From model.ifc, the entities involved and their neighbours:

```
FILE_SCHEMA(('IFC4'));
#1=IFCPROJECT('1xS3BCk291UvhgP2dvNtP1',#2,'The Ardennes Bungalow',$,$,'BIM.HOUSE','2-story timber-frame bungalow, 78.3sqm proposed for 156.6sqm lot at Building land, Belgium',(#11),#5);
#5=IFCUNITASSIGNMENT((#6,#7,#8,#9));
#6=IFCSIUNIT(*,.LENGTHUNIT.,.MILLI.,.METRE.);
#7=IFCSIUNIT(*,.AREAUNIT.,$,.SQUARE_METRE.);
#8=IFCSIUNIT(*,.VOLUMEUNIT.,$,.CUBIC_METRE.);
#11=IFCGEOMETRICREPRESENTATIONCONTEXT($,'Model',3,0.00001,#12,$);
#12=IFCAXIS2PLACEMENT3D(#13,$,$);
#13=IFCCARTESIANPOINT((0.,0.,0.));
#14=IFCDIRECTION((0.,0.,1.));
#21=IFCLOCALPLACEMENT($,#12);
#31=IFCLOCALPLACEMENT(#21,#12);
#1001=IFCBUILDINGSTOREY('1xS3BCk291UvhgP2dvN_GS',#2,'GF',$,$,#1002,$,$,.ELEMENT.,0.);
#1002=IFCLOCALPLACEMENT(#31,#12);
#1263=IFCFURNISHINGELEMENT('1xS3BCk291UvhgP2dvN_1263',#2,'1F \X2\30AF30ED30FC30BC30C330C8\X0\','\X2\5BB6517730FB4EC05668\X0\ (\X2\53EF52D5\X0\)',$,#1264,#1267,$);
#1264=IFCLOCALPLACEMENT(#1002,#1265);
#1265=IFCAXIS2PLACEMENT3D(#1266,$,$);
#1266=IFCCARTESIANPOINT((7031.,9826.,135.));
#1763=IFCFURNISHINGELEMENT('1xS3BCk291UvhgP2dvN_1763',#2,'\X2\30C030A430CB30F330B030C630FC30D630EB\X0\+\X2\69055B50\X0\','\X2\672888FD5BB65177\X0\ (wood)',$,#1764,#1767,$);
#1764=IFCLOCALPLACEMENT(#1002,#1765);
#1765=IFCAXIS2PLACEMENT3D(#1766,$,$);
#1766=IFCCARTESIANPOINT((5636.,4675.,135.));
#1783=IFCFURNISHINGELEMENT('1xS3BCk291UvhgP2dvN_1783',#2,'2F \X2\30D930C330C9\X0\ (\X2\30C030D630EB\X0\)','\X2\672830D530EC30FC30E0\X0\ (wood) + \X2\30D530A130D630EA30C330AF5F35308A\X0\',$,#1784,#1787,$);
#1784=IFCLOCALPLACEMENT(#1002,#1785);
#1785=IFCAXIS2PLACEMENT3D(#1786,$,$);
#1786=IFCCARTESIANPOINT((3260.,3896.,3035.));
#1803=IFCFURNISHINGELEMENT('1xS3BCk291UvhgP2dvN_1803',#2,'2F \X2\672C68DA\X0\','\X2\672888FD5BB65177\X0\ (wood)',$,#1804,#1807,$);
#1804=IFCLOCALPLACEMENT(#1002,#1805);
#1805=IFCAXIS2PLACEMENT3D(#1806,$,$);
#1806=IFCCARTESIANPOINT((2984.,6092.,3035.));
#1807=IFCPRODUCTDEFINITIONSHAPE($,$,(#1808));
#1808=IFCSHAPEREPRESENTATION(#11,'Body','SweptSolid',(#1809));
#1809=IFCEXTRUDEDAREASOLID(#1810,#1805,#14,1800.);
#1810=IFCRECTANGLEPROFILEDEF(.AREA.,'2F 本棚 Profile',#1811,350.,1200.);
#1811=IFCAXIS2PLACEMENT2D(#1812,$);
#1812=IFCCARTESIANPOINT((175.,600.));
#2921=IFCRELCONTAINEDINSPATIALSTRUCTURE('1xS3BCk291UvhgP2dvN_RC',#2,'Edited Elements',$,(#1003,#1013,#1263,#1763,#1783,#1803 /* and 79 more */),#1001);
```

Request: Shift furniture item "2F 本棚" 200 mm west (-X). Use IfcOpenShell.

```python
import ifcopenshell
import ifcopenshell.api.geometry
import ifcopenshell.util.placement
import ifcopenshell.util.unit

model = ifcopenshell.open("model.ifc")
unit_scale = ifcopenshell.util.unit.calculate_unit_scale(model)

item = model.by_guid("1xS3BCk291UvhgP2dvN_1803")
matrix = ifcopenshell.util.placement.get_local_placement(item.ObjectPlacement)
matrix[0, 3] -= 0.2 / unit_scale
ifcopenshell.api.geometry.edit_object_placement(model, product=item, matrix=matrix, is_si=False)

print(ifcopenshell.util.placement.get_local_placement(item.ObjectPlacement).round(3) + 0.0)

model.write("model-out.ifc")
```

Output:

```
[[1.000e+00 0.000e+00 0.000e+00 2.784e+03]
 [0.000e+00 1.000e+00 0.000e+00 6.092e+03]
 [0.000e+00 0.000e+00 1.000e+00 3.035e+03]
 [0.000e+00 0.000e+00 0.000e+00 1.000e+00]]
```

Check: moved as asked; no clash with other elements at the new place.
